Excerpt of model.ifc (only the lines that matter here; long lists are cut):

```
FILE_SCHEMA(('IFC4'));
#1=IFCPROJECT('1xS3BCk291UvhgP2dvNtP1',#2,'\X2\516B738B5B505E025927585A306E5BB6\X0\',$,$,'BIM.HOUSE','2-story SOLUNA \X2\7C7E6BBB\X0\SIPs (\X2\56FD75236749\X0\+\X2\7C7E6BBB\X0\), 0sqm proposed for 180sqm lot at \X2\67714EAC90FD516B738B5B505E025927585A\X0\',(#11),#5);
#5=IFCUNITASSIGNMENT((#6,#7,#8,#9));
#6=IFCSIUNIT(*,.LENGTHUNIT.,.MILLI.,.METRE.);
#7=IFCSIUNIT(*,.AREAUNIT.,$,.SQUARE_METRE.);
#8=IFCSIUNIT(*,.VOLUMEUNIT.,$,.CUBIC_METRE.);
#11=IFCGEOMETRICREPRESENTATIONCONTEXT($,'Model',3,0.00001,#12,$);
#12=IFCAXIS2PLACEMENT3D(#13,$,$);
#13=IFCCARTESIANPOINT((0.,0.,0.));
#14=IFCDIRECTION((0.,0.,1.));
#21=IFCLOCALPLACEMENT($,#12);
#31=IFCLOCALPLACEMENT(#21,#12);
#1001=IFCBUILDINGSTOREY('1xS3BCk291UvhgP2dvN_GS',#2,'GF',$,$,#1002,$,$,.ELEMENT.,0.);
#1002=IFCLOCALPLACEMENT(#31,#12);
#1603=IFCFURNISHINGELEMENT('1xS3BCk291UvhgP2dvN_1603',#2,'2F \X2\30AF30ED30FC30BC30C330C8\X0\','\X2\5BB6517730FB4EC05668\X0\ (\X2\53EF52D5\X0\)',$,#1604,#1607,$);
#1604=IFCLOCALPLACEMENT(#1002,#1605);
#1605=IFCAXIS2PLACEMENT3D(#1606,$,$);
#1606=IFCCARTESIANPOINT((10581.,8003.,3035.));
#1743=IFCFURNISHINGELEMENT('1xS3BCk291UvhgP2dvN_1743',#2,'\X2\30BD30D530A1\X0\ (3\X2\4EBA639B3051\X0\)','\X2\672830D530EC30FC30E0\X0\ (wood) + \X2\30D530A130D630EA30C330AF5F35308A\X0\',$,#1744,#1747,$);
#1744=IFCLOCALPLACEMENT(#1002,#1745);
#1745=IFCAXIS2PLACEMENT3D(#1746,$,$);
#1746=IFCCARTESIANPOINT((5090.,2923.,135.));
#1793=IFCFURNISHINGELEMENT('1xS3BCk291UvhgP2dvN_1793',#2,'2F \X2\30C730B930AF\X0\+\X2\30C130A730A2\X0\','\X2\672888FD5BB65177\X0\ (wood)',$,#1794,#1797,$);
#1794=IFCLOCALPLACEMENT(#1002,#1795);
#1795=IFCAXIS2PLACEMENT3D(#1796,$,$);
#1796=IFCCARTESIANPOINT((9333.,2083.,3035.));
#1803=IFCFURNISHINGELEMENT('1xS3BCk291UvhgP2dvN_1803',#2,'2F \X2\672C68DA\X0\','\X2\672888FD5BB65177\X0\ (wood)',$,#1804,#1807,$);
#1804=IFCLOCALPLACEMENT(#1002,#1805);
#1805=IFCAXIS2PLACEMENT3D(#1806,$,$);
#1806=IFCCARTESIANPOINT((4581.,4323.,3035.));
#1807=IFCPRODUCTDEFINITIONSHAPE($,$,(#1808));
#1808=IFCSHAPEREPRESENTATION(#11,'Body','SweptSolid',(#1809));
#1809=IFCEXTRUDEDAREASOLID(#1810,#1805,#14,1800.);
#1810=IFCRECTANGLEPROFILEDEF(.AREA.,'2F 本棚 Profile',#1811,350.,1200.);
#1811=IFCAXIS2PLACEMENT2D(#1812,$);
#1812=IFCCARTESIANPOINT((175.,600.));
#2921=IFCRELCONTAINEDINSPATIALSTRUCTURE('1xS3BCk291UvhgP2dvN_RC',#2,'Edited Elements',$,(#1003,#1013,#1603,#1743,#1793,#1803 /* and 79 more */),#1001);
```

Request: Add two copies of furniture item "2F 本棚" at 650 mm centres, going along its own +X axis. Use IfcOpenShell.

```python
import ifcopenshell
import ifcopenshell.api.geometry
import ifcopenshell.api.root
import ifcopenshell.util.element
import ifcopenshell.util.placement
import ifcopenshell.util.unit

model = ifcopenshell.open("model.ifc")
unit_scale = ifcopenshell.util.unit.calculate_unit_scale(model)


def reuse_history(source, copy):
    """copy_class also copies each property set's owner history, people and application; keep the originals."""
    for rel in copy.IsDefinedBy:
        if rel.is_a("IfcRelDefinesByProperties") and (history := rel.RelatingPropertyDefinition.OwnerHistory):
            rel.RelatingPropertyDefinition.OwnerHistory = source.OwnerHistory
            ifcopenshell.util.element.remove_deep2(model, history)


source = model.by_id(1803)
base = ifcopenshell.util.placement.get_local_placement(source.ObjectPlacement)
step = base[:3, 0] * 0.65 / unit_scale

for i in range(1, 3):
    copy = ifcopenshell.api.root.copy_class(model, product=source)
    copy.Representation = ifcopenshell.util.element.copy_deep(
        model, source.Representation, exclude=["IfcGeometricRepresentationContext", "IfcRepresentationMap"]
    )
    reuse_history(source, copy)
    matrix = base.copy()
    matrix[:3, 3] += i * step
    print("added at", matrix[:3, 3].round(3) + 0.0)
    ifcopenshell.api.geometry.edit_object_placement(model, product=copy, matrix=matrix, is_si=False)

model.write("model-out.ifc")
```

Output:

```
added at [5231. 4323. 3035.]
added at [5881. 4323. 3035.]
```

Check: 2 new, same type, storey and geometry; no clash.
